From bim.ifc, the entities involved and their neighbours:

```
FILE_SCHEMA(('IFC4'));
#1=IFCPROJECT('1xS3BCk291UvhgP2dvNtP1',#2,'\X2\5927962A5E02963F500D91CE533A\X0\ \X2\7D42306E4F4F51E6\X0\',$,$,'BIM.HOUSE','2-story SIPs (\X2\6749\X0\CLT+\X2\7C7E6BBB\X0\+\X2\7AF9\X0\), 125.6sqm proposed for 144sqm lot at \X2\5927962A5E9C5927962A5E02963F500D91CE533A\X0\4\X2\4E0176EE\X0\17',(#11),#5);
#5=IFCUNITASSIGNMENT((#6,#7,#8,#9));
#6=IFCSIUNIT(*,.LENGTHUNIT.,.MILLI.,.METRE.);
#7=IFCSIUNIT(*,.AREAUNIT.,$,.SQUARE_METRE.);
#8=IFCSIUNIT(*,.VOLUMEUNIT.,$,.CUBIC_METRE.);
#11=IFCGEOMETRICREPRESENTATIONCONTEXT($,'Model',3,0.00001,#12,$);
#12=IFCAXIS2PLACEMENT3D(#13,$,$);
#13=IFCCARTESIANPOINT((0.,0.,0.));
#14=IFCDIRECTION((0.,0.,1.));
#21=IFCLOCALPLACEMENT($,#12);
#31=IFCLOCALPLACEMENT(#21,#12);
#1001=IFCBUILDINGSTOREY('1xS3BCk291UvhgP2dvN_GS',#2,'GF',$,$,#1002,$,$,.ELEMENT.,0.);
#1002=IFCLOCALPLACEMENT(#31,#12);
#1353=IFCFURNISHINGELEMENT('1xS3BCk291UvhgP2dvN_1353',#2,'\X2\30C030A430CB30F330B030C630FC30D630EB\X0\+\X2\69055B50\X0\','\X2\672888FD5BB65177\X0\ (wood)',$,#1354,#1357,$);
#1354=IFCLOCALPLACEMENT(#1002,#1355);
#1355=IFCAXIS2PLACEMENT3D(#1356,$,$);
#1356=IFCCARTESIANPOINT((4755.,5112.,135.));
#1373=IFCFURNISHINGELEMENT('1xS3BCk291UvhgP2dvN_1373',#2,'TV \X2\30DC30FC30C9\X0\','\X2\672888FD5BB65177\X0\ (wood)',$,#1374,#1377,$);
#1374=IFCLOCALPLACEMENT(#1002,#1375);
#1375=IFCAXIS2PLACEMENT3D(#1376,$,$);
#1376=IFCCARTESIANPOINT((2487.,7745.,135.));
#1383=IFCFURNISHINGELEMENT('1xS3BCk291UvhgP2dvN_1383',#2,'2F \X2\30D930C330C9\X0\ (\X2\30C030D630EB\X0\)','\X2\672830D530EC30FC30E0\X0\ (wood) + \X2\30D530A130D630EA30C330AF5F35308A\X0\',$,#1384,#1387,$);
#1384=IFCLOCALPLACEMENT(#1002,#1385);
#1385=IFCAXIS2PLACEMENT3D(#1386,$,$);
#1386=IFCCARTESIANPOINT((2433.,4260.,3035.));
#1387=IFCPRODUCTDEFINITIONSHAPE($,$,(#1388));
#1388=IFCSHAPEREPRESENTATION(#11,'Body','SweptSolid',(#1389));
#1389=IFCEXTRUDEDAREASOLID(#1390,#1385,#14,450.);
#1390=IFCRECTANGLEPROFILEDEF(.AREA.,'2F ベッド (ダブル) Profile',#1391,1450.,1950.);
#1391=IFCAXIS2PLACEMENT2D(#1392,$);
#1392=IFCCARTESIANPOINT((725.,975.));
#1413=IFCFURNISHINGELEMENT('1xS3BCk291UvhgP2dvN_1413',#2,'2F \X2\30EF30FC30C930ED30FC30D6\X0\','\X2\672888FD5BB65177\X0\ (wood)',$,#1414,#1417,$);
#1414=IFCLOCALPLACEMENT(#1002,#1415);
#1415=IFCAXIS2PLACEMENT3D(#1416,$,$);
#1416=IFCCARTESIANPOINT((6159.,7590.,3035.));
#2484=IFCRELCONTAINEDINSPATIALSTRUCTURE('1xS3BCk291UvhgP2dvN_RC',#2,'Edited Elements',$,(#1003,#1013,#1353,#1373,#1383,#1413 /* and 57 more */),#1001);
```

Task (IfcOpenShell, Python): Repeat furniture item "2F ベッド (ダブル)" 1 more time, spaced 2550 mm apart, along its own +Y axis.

```python
import ifcopenshell
import ifcopenshell.api.geometry
import ifcopenshell.api.root
import ifcopenshell.util.element
import ifcopenshell.util.placement
import ifcopenshell.util.unit

model = ifcopenshell.open("bim.ifc")
unit_scale = ifcopenshell.util.unit.calculate_unit_scale(model)


def reuse_history(source, copy):
    """copy_class also copies each property set's owner history, people and application; keep the originals."""
    for rel in copy.IsDefinedBy:
        if rel.is_a("IfcRelDefinesByProperties") and (history := rel.RelatingPropertyDefinition.OwnerHistory):
            rel.RelatingPropertyDefinition.OwnerHistory = source.OwnerHistory
            ifcopenshell.util.element.remove_deep2(model, history)


source = model.by_guid("1xS3BCk291UvhgP2dvN_1383")
base = ifcopenshell.util.placement.get_local_placement(source.ObjectPlacement)
step = base[:3, 1] * 2.55 / unit_scale

for i in range(1, 2):
    copy = ifcopenshell.api.root.copy_class(model, product=source)
    copy.Representation = ifcopenshell.util.element.copy_deep(
        model, source.Representation, exclude=["IfcGeometricRepresentationContext", "IfcRepresentationMap"]
    )
    reuse_history(source, copy)
    matrix = base.copy()
    matrix[:3, 3] += i * step
    print("added at", matrix[:3, 3].round(3) + 0.0)
    ifcopenshell.api.geometry.edit_object_placement(model, product=copy, matrix=matrix, is_si=False)

model.write("bim_rev.ifc")
```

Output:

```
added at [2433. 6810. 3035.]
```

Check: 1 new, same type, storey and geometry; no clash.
